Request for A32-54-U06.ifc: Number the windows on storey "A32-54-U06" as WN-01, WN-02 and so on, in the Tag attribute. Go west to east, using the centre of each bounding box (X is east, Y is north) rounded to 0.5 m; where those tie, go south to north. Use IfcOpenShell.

First a look at what the model holds.

```python
import ifcopenshell
import ifcopenshell.util.element
import ifcopenshell.util.placement

model = ifcopenshell.open("A32-54-U06.ifc")
print(model.schema)
storey = next(s for s in model.by_type("IfcBuildingStorey") if s.Name == "A32-54-U06")
windows = [e for e in ifcopenshell.util.element.get_decomposition(storey) if e.is_a("IfcWindow")]
for e in sorted(windows, key=lambda e: e.id()):
    origin = ifcopenshell.util.placement.get_local_placement(e.ObjectPlacement)[:3, 3]
    print(e.id(), e.Tag, e.Name, origin.round(2) + 0.0, sep=" | ")
```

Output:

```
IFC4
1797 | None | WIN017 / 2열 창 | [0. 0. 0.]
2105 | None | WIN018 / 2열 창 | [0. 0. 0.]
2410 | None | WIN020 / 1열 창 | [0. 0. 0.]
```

```python
import ifcopenshell
import ifcopenshell.geom
import ifcopenshell.util.element
import ifcopenshell.util.shape

model = ifcopenshell.open("A32-54-U06.ifc")
settings = ifcopenshell.geom.settings()
settings.set("use-world-coords", True)


def centre(element):
    shape = ifcopenshell.geom.create_shape(settings, element)
    return ifcopenshell.util.shape.get_bbox_centroid(shape.geometry)


storey = next(s for s in model.by_type("IfcBuildingStorey") if s.Name == "A32-54-U06")
windows = [e for e in ifcopenshell.util.element.get_decomposition(storey) if e.is_a("IfcWindow")]

# Insertion points can sit at a corner or the storey origin, so sort by the geometry (in metres).
centres = {e: centre(e) for e in windows}
windows.sort(key=lambda e: (round(centres[e][0] / 0.5), centres[e][1]))

for i, e in enumerate(windows, start=1):
    number = f"WN-{i:02d}"
    e.Tag = number
    print(e.id(), number)

model.write("A32-54-U06_rev.ifc")
```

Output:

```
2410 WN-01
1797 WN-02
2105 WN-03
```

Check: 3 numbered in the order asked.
